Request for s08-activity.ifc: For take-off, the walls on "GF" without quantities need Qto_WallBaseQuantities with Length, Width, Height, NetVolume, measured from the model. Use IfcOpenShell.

First a look at what the model holds.

```python
import ifcopenshell
import ifcopenshell.util.element
import ifcopenshell.util.unit

model = ifcopenshell.open("s08-activity.ifc")
print(model.schema)
for unit_type in ("LENGTHUNIT", "AREAUNIT", "VOLUMEUNIT"):
    print(unit_type, ifcopenshell.util.unit.calculate_unit_scale(model, unit_type))
storey = next(s for s in model.by_type("IfcBuildingStorey") if s.Name == "GF")
walls = [e for e in ifcopenshell.util.element.get_decomposition(storey) if e.is_a("IfcWall")]
for e in sorted(walls, key=lambda e: e.id()):
    print(e.id(), e.is_a(), e.Name, list(ifcopenshell.util.element.get_psets(e, qtos_only=True)), sep=" | ")
```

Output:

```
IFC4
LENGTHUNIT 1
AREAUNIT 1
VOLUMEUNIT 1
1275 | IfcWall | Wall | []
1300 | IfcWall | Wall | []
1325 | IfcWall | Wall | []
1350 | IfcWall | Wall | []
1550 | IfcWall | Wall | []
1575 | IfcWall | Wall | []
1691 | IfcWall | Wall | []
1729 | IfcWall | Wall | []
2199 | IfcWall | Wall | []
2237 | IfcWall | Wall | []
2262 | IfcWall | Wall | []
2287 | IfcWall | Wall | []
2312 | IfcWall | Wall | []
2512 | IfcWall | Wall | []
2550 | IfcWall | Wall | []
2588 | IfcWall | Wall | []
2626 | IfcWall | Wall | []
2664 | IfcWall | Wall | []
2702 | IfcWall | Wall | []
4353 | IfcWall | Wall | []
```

```python
import ifcopenshell
import ifcopenshell.api.pset
import ifcopenshell.geom
import ifcopenshell.util.element
import ifcopenshell.util.shape
import ifcopenshell.util.unit

model = ifcopenshell.open("s08-activity.ifc")
unit_scale = ifcopenshell.util.unit.calculate_unit_scale(model)
volume_scale = ifcopenshell.util.unit.calculate_unit_scale(model, "VOLUMEUNIT")
settings = ifcopenshell.geom.settings()

storey = next(s for s in model.by_type("IfcBuildingStorey") if s.Name == "GF")
walls = [e for e in ifcopenshell.util.element.get_decomposition(storey) if e.is_a("IfcWall")]

for e in sorted(walls, key=lambda e: e.id()):
    if ifcopenshell.util.element.get_psets(e, qtos_only=True, should_inherit=False):
        continue
    # Geometry comes back in metres, in the element's own axes.
    shape = ifcopenshell.geom.create_shape(settings, e)
    values = {
        "Length": ifcopenshell.util.shape.get_x(shape.geometry) / unit_scale,
        "Width": ifcopenshell.util.shape.get_y(shape.geometry) / unit_scale,
        "Height": ifcopenshell.util.shape.get_z(shape.geometry) / unit_scale,
        "NetVolume": ifcopenshell.util.shape.get_volume(shape.geometry) / volume_scale,
    }
    qto = ifcopenshell.api.pset.add_qto(model, product=e, name="Qto_WallBaseQuantities")
    ifcopenshell.api.pset.edit_qto(model, qto=qto, properties=values)
    print(e.id(), {k: round(v, 3) for k, v in values.items()})

model.write("s08-activity_rev.ifc")
```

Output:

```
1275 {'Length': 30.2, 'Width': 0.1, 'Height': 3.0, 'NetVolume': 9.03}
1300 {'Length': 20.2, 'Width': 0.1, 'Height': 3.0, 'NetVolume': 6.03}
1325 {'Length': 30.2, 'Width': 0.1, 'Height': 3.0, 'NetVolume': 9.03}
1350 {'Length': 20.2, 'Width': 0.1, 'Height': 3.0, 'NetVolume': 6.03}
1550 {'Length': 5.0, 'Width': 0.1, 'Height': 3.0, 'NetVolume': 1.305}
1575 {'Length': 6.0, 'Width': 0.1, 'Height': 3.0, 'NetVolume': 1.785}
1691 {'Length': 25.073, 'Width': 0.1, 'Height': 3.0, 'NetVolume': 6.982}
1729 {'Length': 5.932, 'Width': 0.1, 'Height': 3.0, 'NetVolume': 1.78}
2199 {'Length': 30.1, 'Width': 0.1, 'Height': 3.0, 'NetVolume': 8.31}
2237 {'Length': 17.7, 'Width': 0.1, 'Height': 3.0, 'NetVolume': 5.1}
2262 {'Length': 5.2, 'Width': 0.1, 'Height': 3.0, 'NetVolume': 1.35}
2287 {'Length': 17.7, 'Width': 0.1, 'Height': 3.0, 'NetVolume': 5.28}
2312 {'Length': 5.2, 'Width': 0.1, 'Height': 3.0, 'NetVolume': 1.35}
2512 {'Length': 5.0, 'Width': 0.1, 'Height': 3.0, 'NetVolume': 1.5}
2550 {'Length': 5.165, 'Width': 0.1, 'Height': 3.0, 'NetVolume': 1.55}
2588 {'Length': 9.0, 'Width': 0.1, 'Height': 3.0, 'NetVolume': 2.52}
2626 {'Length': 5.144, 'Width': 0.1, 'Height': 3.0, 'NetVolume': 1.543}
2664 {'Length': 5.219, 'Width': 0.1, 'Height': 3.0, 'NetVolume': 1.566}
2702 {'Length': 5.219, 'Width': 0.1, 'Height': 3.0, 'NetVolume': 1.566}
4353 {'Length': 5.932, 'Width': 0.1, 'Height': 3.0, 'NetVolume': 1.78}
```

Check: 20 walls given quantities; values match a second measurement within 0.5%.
